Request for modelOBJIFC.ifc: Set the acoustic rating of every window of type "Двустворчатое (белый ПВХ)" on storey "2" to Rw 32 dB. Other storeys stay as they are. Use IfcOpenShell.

First a look at what the model holds.

```python
import ifcopenshell
import ifcopenshell.util.element

model = ifcopenshell.open("modelOBJIFC.ifc")
print(model.schema)
storey = next(s for s in model.by_type("IfcBuildingStorey") if s.Name == "2")
windows = [e for e in ifcopenshell.util.element.get_decomposition(storey) if e.is_a("IfcWindow")]
seen = {}
for e in windows:
    element_type = ifcopenshell.util.element.get_type(e)
    key = (element_type.Name if element_type != e and element_type else None, ifcopenshell.util.element.get_pset(e, "Pset_WindowCommon", "AcousticRating"))
    seen[key] = seen.get(key, 0) + 1
for (name, value), count in sorted(seen.items(), key=str):
    print(count, "x", name, "|", value)
```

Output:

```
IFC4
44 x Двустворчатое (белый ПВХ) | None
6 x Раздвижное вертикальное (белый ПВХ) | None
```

```python
import ifcopenshell
import ifcopenshell.api.pset
import ifcopenshell.util.element

model = ifcopenshell.open("modelOBJIFC.ifc")

storey = next(s for s in model.by_type("IfcBuildingStorey") if s.Name == "2")
windows = [e for e in ifcopenshell.util.element.get_decomposition(storey) if e.is_a("IfcWindow")]

count = 0
for e in windows:
    element_type = ifcopenshell.util.element.get_type(e)
    if element_type in (None, e) or element_type.Name != "Двустворчатое (белый ПВХ)":
        continue
    # add_pset returns the element's existing set when there is one.
    pset = ifcopenshell.api.pset.add_pset(model, product=e, name="Pset_WindowCommon")
    ifcopenshell.api.pset.edit_pset(model, pset=pset, properties={"AcousticRating": "Rw 32 dB"})
    count += 1

print(count, "windows updated")

model.write("modelOBJIFC_updated.ifc")
```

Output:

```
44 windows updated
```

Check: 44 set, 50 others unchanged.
